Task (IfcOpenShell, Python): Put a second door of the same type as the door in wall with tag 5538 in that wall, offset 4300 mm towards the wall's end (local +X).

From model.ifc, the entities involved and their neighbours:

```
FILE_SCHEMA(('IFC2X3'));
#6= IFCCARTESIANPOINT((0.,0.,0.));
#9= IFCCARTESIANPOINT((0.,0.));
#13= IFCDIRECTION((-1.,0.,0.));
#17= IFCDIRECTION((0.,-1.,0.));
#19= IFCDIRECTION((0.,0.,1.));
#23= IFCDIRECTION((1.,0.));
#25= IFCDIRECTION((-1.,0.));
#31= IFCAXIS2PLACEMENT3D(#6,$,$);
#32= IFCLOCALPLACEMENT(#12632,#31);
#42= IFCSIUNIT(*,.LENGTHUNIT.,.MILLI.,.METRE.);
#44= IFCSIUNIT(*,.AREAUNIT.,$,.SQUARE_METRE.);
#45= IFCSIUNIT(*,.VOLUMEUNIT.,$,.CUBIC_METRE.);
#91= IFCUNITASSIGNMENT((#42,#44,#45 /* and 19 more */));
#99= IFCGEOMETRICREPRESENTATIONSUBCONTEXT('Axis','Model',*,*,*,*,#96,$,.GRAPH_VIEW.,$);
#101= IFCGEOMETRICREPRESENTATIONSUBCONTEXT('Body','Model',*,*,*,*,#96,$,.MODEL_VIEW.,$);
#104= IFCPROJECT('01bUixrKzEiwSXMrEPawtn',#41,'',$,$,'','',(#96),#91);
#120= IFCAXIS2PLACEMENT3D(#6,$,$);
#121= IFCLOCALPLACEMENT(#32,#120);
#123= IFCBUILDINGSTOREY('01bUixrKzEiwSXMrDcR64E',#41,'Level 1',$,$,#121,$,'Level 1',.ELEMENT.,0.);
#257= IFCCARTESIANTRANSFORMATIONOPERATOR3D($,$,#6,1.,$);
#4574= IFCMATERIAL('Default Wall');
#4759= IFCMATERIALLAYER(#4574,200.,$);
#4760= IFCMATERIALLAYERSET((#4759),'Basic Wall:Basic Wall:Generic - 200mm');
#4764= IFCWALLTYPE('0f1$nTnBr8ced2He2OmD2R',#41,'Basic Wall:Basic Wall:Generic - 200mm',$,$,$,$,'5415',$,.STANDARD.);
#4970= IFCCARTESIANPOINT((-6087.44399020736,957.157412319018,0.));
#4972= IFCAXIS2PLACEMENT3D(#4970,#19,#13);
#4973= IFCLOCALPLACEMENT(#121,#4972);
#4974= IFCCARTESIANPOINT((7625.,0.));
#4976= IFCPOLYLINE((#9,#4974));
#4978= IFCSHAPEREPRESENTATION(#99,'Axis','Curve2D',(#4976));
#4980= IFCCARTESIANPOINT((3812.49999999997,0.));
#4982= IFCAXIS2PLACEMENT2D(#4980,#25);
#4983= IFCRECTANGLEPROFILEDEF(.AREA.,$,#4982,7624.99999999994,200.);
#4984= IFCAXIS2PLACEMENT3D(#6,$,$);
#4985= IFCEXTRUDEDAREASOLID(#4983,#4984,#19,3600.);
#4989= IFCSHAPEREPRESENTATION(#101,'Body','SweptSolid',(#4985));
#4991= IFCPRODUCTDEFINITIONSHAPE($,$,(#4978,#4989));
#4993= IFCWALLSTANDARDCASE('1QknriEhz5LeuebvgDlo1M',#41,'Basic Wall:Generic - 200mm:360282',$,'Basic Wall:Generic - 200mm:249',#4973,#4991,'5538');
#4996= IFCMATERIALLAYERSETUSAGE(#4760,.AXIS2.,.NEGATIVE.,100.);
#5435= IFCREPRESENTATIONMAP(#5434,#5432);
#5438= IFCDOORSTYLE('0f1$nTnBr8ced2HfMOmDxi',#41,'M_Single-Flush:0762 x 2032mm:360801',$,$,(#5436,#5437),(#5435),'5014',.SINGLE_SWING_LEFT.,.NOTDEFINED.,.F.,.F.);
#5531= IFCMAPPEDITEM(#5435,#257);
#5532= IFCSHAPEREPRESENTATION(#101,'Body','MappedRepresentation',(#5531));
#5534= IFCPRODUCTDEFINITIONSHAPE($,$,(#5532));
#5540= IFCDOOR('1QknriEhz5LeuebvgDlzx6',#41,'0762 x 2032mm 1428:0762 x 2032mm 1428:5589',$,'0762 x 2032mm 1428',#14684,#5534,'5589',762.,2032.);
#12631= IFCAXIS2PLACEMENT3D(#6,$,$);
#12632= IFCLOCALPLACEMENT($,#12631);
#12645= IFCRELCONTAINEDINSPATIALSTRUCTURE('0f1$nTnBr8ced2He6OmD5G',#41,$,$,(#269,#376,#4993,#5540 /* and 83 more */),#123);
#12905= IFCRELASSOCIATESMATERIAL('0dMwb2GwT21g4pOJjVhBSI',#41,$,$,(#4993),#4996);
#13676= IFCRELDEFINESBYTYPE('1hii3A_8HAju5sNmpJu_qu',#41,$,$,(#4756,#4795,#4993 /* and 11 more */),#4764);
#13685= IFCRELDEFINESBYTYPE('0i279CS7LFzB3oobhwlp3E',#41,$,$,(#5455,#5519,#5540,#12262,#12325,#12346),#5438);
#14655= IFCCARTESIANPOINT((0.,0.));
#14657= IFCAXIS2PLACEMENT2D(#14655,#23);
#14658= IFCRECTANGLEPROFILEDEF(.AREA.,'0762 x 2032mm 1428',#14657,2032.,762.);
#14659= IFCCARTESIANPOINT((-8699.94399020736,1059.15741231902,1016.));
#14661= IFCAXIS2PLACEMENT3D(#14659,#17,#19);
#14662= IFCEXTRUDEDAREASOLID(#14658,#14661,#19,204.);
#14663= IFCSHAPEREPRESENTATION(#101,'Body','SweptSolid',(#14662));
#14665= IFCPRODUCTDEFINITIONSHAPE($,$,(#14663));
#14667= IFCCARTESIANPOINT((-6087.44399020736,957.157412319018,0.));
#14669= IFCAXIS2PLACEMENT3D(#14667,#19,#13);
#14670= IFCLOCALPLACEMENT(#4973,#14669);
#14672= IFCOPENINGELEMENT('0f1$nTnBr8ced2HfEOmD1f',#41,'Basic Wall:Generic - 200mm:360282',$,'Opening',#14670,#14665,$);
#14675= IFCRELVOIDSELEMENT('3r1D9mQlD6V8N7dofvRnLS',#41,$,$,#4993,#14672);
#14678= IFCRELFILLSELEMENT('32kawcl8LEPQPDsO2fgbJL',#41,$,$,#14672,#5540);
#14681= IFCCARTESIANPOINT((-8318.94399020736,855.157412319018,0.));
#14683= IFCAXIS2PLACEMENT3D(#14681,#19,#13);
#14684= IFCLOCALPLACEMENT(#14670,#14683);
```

```python
import ifcopenshell
import ifcopenshell.api.feature
import ifcopenshell.api.geometry
import ifcopenshell.api.root
import ifcopenshell.geom
import ifcopenshell.util.element
import ifcopenshell.util.placement
import ifcopenshell.util.shape

model = ifcopenshell.open("model.ifc")
settings = ifcopenshell.geom.settings()


def volume(element):
    """Net volume in cubic metres, openings subtracted."""
    shape = ifcopenshell.geom.create_shape(settings, element)
    return ifcopenshell.util.shape.get_volume(shape.geometry)


def reuse_history(source, copy):
    """copy_class also copies each property set's owner history, people and application; keep the originals."""
    for rel in copy.IsDefinedBy:
        if rel.is_a("IfcRelDefinesByProperties") and (history := rel.RelatingPropertyDefinition.OwnerHistory):
            rel.RelatingPropertyDefinition.OwnerHistory = source.OwnerHistory
            ifcopenshell.util.element.remove_deep2(model, history)


door = model.by_guid("1QknriEhz5LeuebvgDlzx6")
opening = door.FillsVoids[0].RelatingOpeningElement
wall = opening.VoidsElements[0].RelatingBuildingElement
before = volume(wall)
shift = ifcopenshell.util.placement.get_local_placement(wall.ObjectPlacement)[:3, 0] * 4300.0

# copy_class copies the void relationship, type, container and properties, but no geometry.
new_opening = ifcopenshell.api.root.copy_class(model, product=opening)
new_opening.Representation = ifcopenshell.util.element.copy_deep(
    model, opening.Representation, exclude=["IfcGeometricRepresentationContext", "IfcRepresentationMap"]
)
new_opening.Name = "Basic Wall:Generic - 200mm"
new_door = ifcopenshell.api.root.copy_class(model, product=door)
new_door.Representation = ifcopenshell.util.element.copy_deep(
    model, door.Representation, exclude=["IfcGeometricRepresentationContext", "IfcRepresentationMap"]
)
new_door.Name = "0762 x 2032mm 1428:0762 x 2032mm 1428"
new_door.Tag = None
reuse_history(door, new_door)
fills = ifcopenshell.api.feature.add_filling(model, opening=new_opening, element=new_door)
fills.OwnerHistory = new_door.OwnerHistory  # required in IFC2X3

for old, new in ((opening, new_opening), (door, new_door)):
    matrix = ifcopenshell.util.placement.get_local_placement(old.ObjectPlacement)
    matrix[:3, 3] += shift
    ifcopenshell.api.geometry.edit_object_placement(model, product=new, matrix=matrix, is_si=False)

after = volume(wall)

print(f"wall volume {before:.3f} -> {after:.3f} m3")

model.write("model-out.ifc")
```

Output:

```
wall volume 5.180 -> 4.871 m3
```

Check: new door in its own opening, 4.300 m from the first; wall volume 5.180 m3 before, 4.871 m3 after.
